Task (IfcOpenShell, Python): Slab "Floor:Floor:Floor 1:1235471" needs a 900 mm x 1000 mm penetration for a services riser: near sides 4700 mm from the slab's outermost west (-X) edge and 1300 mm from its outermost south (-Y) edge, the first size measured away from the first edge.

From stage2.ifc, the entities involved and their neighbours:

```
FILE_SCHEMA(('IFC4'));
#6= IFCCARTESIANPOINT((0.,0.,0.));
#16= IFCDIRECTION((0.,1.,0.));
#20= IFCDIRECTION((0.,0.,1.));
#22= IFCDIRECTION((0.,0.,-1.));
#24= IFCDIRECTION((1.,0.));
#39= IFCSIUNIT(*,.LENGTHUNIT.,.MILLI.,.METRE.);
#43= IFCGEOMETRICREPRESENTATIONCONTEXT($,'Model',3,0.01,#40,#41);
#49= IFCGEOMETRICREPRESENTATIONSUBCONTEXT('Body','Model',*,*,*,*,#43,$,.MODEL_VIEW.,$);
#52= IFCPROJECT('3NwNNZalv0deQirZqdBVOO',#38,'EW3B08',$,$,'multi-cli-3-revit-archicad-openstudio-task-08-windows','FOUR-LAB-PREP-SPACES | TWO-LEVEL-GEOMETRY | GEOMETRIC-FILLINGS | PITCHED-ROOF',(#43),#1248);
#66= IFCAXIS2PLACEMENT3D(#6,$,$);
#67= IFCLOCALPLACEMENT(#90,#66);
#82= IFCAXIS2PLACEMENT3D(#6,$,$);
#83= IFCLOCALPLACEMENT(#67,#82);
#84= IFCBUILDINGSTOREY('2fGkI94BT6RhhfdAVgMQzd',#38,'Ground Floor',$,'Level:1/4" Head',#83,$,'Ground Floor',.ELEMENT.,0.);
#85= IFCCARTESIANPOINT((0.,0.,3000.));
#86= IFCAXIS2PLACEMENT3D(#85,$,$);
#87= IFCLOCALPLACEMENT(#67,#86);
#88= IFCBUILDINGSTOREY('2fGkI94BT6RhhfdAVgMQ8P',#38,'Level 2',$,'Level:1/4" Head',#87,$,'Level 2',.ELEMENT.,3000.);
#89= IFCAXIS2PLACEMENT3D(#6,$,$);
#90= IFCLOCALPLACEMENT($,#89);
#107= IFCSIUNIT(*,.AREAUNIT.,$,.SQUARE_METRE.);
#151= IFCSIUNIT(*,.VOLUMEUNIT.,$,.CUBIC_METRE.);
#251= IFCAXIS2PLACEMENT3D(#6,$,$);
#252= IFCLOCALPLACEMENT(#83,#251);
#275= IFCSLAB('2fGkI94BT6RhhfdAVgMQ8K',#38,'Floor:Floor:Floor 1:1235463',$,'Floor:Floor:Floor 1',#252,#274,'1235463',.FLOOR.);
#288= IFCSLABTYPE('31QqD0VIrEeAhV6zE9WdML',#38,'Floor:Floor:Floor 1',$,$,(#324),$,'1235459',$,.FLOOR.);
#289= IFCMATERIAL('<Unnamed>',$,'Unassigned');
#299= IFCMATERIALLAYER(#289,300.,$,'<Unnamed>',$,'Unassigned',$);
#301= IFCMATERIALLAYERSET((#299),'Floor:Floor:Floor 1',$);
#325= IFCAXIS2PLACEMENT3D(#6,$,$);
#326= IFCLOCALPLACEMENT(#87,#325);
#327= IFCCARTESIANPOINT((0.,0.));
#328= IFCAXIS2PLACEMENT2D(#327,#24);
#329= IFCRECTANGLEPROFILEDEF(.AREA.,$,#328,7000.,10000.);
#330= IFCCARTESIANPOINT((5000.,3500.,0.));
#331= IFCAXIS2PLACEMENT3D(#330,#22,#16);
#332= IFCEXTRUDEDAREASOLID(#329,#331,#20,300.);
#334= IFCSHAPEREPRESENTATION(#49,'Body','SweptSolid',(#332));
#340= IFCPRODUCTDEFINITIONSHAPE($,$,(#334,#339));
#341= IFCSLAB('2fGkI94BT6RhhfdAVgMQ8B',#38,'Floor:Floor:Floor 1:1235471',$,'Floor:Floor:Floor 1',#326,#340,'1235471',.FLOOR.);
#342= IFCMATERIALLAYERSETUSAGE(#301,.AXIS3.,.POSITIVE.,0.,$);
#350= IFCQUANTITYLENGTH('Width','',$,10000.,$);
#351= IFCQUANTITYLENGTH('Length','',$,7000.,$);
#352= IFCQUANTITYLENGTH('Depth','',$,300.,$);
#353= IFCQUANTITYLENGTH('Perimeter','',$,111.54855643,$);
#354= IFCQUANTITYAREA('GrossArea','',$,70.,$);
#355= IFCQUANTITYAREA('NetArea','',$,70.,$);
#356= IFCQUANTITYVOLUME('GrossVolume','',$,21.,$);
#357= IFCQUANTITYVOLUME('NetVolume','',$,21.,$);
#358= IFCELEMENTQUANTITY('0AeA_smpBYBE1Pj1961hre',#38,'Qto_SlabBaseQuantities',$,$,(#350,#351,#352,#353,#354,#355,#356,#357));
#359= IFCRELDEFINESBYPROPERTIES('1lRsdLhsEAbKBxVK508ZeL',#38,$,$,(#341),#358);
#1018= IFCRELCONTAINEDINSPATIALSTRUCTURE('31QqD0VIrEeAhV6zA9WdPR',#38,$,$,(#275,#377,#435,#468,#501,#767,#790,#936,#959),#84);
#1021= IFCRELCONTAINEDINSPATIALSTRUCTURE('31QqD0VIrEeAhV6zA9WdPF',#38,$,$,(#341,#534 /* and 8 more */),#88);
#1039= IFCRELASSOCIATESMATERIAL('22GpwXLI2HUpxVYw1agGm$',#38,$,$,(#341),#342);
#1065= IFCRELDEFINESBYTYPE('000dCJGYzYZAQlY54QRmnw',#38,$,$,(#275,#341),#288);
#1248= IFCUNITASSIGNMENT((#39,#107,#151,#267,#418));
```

```python
import numpy as np
import ifcopenshell
import ifcopenshell.api.feature
import ifcopenshell.api.geometry
import ifcopenshell.api.pset
import ifcopenshell.api.root
import ifcopenshell.geom
import ifcopenshell.util.element
import ifcopenshell.util.placement
import ifcopenshell.util.representation
import ifcopenshell.util.shape
import ifcopenshell.util.unit

model = ifcopenshell.open("stage2.ifc")
unit_scale = ifcopenshell.util.unit.calculate_unit_scale(model)
area_scale = ifcopenshell.util.unit.calculate_unit_scale(model, "AREAUNIT")
volume_scale = ifcopenshell.util.unit.calculate_unit_scale(model, "VOLUMEUNIT")
settings = ifcopenshell.geom.settings()


def volume(element):
    """Net volume in cubic metres, openings subtracted."""
    shape = ifcopenshell.geom.create_shape(settings, element)
    return ifcopenshell.util.shape.get_volume(shape.geometry)


slab = model.by_guid("2fGkI94BT6RhhfdAVgMQ8B")
before = volume(slab)

# Extent in the slab's own axes, in metres. The edges named are its -X and -Y sides.
slab_shape = ifcopenshell.geom.create_shape(settings, slab)
vertices = ifcopenshell.util.shape.get_vertices(slab_shape.geometry)
x_min, y_min, bottom = vertices.min(axis=0)
top = vertices[:, 2].max()

opening = ifcopenshell.api.root.create_entity(model, ifc_class="IfcOpeningElement", name="Services riser opening", predefined_type="OPENING")
context = ifcopenshell.util.representation.get_context(model, "Model", "Body", "MODEL_VIEW")
width, depth = 0.9, 1
outline = [(0.0, 0.0), (width, 0.0), (width, depth), (0.0, depth), (0.0, 0.0)]
# Overshoot both faces by 50 mm so the cut is clean.
shape = ifcopenshell.api.geometry.add_slab_representation(
    model, context=context, depth=top - bottom + 0.1, polyline=outline
)
ifcopenshell.api.geometry.assign_representation(model, product=opening, representation=shape)

matrix = ifcopenshell.util.placement.get_local_placement(slab.ObjectPlacement)
matrix[:, 3] = matrix @ np.append(np.array([x_min + 4.7, y_min + 1.3, bottom - 0.05]) / unit_scale, 1.0)
ifcopenshell.api.geometry.edit_object_placement(model, product=opening, matrix=matrix, is_si=False)
ifcopenshell.api.feature.add_feature(model, feature=opening, element=slab)

after = volume(slab)

# Update the slab's stored quantities.
qto = model.by_id(ifcopenshell.util.element.get_pset(slab, "Qto_SlabBaseQuantities", should_inherit=False)["id"])
ifcopenshell.api.pset.edit_qto(model, qto=qto, properties={
    "NetArea": after / (top - bottom) / area_scale,
    "NetVolume": after / volume_scale,
})

print(f"slab volume {before:.3f} -> {after:.3f} m3")

model.write("stage2_updated.ifc")
```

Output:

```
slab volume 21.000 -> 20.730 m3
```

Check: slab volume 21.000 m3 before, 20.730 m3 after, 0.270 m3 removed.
